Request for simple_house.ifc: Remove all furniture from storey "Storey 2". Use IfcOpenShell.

First a look at what the model holds.

```python
import ifcopenshell
import ifcopenshell.util.element

model = ifcopenshell.open("simple_house.ifc")
print(model.schema)
storey = next(s for s in model.by_type("IfcBuildingStorey") if s.Name == "Storey 2")
furniture = [e for e in ifcopenshell.util.element.get_decomposition(storey) if e.is_a("IfcFurnishingElement")]
seen = {}
for e in furniture:
    element_type = ifcopenshell.util.element.get_type(e)
    name = element_type.Name if element_type not in (None, e) else None
    seen[name] = seen.get(name, 0) + 1
for name, count in sorted(seen.items(), key=str):
    print(count, "x", name)
```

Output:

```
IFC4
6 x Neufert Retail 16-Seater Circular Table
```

```python
import ifcopenshell
import ifcopenshell.api.root
import ifcopenshell.util.element

model = ifcopenshell.open("simple_house.ifc")

storey = next(s for s in model.by_type("IfcBuildingStorey") if s.Name == "Storey 2")
furniture = [e for e in ifcopenshell.util.element.get_decomposition(storey) if e.is_a("IfcFurnishingElement")]

for e in furniture:
    ifcopenshell.api.root.remove_product(model, product=e)
print(len(furniture), "removed")

model.write("simple_house_rev.ifc")
```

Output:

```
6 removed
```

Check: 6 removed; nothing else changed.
